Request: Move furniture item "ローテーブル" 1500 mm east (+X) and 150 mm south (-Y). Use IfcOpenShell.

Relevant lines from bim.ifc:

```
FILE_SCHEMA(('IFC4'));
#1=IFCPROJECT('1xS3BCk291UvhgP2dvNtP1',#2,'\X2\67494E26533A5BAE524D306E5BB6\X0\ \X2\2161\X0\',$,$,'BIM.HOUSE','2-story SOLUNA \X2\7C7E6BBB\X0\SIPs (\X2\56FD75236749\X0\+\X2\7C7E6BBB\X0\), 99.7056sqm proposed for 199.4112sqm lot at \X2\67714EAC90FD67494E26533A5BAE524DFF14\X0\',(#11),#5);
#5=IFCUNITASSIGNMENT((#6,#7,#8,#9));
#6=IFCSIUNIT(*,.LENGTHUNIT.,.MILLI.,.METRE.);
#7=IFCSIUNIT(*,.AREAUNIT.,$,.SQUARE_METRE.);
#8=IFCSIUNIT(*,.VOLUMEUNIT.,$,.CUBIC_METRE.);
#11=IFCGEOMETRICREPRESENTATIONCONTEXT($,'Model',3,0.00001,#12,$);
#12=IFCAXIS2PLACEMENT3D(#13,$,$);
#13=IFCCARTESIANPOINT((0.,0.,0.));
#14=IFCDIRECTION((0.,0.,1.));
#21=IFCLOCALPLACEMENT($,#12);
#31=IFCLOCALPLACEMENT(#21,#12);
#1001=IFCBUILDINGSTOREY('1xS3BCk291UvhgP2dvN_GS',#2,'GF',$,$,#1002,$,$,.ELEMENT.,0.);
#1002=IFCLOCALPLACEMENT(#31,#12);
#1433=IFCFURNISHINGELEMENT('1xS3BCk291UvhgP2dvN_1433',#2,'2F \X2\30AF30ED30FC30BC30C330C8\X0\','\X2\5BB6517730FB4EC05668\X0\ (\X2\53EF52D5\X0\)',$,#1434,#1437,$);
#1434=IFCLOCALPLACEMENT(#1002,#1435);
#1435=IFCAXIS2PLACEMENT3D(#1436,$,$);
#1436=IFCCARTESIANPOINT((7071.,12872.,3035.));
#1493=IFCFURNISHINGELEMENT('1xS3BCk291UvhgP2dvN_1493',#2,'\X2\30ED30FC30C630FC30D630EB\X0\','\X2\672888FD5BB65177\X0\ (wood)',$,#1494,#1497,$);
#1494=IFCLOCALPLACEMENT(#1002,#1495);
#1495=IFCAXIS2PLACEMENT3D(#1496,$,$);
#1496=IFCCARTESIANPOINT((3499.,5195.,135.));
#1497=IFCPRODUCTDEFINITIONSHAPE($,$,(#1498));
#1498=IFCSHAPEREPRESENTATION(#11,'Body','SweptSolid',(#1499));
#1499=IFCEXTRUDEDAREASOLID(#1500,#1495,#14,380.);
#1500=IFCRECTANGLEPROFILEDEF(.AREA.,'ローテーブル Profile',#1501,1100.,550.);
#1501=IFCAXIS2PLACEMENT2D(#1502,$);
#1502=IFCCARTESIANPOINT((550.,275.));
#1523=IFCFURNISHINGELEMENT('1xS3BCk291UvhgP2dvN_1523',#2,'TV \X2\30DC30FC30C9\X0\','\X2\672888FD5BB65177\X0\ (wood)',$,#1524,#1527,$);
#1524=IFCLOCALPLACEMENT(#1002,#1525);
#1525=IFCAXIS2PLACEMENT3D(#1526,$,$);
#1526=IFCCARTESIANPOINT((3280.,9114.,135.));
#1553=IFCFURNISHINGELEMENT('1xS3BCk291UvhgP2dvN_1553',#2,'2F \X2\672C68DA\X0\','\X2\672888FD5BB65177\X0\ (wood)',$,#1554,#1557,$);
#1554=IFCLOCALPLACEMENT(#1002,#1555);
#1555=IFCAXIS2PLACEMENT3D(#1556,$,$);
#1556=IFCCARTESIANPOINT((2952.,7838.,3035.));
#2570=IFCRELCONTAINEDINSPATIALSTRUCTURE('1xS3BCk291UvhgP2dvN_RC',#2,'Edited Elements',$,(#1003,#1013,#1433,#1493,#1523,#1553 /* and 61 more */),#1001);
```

```python
import ifcopenshell
import ifcopenshell.api.geometry
import ifcopenshell.util.placement

model = ifcopenshell.open("bim.ifc")

item = model.by_guid("1xS3BCk291UvhgP2dvN_1493")
matrix = ifcopenshell.util.placement.get_local_placement(item.ObjectPlacement)
matrix[0, 3] += 1500.0
matrix[1, 3] -= 150.0
ifcopenshell.api.geometry.edit_object_placement(model, product=item, matrix=matrix, is_si=False)

print(ifcopenshell.util.placement.get_local_placement(item.ObjectPlacement).round(3) + 0.0)

model.write("bim-out.ifc")
```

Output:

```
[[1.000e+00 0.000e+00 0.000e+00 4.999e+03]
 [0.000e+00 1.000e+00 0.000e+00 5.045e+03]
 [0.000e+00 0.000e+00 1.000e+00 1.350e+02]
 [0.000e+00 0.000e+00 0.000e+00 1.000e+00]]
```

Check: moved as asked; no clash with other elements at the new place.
